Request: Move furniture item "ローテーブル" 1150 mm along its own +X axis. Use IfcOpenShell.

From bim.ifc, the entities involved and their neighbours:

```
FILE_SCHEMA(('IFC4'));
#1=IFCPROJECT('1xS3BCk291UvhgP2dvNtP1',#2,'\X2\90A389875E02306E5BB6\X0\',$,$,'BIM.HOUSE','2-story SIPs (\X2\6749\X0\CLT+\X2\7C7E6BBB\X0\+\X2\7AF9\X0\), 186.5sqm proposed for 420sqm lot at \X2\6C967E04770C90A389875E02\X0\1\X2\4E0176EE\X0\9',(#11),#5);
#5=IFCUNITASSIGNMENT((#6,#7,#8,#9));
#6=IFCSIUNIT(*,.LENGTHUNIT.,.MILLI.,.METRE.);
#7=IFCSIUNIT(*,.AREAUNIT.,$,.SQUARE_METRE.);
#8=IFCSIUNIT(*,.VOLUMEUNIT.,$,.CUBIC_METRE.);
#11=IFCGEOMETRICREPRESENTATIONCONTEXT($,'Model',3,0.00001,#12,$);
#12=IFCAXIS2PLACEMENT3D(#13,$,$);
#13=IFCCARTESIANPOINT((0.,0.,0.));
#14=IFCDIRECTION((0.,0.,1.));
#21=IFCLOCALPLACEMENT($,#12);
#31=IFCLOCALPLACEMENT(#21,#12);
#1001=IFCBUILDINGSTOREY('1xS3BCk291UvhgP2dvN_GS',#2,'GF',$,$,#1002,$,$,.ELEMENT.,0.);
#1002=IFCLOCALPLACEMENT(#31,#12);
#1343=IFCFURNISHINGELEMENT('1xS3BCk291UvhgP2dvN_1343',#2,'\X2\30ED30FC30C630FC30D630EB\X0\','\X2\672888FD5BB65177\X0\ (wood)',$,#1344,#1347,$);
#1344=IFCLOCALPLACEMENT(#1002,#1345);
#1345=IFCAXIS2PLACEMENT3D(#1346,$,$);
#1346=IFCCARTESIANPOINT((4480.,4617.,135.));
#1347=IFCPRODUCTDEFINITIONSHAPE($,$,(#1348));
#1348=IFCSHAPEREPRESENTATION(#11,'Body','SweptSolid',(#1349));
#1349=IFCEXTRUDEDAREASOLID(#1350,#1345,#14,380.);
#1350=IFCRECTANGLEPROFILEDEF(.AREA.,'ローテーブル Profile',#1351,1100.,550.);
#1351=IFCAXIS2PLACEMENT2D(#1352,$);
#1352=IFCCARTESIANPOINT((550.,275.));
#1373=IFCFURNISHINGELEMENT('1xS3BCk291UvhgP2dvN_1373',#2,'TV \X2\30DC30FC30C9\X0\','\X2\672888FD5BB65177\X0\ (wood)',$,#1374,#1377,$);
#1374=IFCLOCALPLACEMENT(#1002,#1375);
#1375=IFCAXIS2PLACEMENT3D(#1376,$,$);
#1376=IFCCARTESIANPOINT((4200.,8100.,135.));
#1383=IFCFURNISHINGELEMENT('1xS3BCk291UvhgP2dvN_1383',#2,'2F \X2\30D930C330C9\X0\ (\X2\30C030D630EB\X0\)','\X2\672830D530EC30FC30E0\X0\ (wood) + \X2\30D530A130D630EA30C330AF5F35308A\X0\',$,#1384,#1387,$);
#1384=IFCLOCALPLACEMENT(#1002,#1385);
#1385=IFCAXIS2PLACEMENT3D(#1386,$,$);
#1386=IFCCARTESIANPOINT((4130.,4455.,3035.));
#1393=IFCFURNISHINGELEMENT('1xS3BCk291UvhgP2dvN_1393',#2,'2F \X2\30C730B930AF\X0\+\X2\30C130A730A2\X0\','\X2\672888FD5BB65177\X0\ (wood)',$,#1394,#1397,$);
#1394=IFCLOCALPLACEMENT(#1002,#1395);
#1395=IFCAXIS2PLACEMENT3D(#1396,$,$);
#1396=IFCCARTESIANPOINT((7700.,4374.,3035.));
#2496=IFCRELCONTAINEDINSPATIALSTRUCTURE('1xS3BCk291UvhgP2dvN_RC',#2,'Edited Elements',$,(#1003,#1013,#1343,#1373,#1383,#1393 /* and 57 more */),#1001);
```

```python
import ifcopenshell
import ifcopenshell.api.geometry
import ifcopenshell.util.placement

model = ifcopenshell.open("bim.ifc")

item = model.by_id(1343)
matrix = ifcopenshell.util.placement.get_local_placement(item.ObjectPlacement)
matrix[:3, 3] += matrix[:3, 0] * 1150.0
ifcopenshell.api.geometry.edit_object_placement(model, product=item, matrix=matrix, is_si=False)

print(ifcopenshell.util.placement.get_local_placement(item.ObjectPlacement).round(3) + 0.0)

model.write("bim_v2.ifc")
```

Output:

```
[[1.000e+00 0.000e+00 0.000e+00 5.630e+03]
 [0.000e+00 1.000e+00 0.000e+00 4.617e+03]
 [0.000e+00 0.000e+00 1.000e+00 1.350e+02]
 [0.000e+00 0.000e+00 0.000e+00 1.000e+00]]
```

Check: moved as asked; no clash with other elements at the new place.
